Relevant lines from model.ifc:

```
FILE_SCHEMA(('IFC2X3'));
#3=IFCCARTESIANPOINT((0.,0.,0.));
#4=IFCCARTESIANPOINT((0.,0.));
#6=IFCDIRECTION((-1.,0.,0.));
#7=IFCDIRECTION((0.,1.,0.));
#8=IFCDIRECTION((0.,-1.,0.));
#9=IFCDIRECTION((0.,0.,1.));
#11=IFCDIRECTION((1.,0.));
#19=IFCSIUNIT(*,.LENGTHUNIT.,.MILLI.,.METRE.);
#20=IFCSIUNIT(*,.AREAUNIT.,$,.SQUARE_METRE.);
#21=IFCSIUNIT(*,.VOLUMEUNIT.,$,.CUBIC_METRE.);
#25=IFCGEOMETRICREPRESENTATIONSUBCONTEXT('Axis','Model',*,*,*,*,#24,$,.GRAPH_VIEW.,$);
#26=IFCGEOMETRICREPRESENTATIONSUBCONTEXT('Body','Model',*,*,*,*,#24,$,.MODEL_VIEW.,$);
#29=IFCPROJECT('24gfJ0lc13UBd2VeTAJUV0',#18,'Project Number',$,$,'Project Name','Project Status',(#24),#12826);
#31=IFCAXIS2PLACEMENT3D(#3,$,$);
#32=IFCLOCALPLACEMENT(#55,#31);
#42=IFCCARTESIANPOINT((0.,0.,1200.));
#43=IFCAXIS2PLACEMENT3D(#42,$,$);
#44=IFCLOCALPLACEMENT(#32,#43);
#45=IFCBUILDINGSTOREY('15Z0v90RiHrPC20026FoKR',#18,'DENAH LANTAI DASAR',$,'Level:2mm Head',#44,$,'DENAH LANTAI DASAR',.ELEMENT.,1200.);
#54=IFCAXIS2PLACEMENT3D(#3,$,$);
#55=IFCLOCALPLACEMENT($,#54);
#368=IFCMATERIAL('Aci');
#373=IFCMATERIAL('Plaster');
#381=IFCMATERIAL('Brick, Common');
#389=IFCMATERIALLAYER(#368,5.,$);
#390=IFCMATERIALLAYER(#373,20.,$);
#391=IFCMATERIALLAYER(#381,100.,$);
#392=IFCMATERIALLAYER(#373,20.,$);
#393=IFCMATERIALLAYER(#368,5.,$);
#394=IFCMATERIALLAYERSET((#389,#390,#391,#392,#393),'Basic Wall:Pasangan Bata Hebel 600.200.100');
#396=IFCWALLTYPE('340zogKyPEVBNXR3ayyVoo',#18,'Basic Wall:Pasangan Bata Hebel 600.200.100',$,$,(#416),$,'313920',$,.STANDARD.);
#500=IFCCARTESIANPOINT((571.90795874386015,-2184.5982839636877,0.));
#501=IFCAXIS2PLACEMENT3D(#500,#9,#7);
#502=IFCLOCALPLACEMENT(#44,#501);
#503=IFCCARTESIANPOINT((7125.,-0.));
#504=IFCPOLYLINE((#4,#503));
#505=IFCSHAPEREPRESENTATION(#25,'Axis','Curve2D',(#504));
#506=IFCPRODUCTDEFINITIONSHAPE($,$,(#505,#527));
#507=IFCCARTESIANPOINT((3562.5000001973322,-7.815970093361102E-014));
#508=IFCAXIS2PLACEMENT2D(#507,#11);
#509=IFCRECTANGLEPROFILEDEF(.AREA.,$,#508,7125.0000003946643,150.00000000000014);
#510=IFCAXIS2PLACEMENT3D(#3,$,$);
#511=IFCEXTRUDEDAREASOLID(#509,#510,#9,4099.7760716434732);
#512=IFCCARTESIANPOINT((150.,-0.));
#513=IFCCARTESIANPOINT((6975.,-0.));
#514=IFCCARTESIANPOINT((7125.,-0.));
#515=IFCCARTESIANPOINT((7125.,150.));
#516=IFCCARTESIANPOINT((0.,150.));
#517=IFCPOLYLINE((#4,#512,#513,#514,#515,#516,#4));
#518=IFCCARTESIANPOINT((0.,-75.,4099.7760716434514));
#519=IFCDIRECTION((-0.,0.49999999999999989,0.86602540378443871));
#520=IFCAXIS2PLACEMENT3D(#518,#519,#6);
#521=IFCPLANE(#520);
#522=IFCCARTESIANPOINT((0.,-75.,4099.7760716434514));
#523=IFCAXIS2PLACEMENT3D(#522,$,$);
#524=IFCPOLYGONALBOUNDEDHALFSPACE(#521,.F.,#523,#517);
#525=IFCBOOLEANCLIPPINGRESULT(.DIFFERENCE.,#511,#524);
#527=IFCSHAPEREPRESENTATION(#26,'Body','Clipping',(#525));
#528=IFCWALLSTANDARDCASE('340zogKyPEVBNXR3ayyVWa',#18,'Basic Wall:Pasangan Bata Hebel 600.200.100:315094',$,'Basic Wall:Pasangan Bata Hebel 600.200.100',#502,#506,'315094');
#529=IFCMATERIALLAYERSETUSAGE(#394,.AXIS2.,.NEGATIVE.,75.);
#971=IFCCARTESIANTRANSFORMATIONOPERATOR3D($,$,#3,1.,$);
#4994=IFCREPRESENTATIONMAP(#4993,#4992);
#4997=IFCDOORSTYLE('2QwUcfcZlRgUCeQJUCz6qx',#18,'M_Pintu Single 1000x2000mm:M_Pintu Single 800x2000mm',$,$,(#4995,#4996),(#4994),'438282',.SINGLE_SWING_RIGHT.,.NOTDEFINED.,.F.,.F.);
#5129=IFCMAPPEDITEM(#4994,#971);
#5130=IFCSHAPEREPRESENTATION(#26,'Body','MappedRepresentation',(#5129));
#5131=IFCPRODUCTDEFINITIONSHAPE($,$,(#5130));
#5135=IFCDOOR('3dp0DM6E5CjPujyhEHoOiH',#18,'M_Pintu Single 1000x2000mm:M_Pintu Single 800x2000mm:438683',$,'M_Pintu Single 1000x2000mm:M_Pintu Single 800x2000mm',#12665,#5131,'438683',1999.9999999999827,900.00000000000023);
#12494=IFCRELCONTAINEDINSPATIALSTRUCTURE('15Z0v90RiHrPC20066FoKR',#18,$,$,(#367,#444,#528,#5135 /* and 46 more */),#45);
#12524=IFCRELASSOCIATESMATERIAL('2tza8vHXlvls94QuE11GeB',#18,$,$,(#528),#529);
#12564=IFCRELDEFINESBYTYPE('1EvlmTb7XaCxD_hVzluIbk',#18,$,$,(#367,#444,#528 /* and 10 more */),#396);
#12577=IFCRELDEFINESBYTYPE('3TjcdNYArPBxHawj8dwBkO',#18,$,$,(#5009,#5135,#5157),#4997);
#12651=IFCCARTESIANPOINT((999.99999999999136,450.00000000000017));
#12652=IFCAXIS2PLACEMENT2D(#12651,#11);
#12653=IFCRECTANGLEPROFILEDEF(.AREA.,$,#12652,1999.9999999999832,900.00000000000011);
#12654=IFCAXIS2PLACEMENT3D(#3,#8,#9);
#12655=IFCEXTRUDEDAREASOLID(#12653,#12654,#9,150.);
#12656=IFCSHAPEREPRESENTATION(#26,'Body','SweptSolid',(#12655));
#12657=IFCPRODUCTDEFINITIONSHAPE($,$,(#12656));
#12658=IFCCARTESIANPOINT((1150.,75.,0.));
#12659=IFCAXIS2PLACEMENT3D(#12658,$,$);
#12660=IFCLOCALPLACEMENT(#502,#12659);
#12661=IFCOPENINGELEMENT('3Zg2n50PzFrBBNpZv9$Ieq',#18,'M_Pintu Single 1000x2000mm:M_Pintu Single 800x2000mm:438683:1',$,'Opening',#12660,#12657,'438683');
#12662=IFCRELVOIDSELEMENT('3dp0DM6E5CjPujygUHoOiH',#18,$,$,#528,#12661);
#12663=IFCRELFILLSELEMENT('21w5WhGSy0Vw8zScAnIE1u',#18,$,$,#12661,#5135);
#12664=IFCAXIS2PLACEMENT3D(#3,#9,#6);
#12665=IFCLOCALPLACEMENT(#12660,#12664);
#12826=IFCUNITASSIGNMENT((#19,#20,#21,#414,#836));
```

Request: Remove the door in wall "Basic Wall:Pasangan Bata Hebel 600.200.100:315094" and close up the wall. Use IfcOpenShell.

```python
import ifcopenshell
import ifcopenshell.api.feature
import ifcopenshell.api.root
import ifcopenshell.geom
import ifcopenshell.util.shape

model = ifcopenshell.open("model.ifc")
settings = ifcopenshell.geom.settings()


def volume(element):
    """Net volume in cubic metres, openings subtracted."""
    shape = ifcopenshell.geom.create_shape(settings, element)
    return ifcopenshell.util.shape.get_volume(shape.geometry)


door = model.by_guid("3dp0DM6E5CjPujyhEHoOiH")
opening = door.FillsVoids[0].RelatingOpeningElement
wall = opening.VoidsElements[0].RelatingBuildingElement
before = volume(wall)

ifcopenshell.api.root.remove_product(model, product=door)
ifcopenshell.api.feature.remove_feature(model, feature=opening)

after = volume(wall)

print(f"wall volume {before:.3f} -> {after:.3f} m3")

model.write("model-out.ifc")
```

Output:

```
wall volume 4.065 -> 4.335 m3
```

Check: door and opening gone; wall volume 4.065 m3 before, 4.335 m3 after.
